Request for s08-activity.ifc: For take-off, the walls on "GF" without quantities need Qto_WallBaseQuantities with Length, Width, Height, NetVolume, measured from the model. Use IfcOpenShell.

First a look at what the model holds.

```python
import ifcopenshell
import ifcopenshell.util.element
import ifcopenshell.util.unit

model = ifcopenshell.open("s08-activity.ifc")
print(model.schema)
for unit_type in ("LENGTHUNIT", "AREAUNIT", "VOLUMEUNIT"):
    print(unit_type, ifcopenshell.util.unit.calculate_unit_scale(model, unit_type))
storey = next(s for s in model.by_type("IfcBuildingStorey") if s.Name == "GF")
walls = [e for e in ifcopenshell.util.element.get_decomposition(storey) if e.is_a("IfcWall")]
for e in sorted(walls, key=lambda e: e.id()):
    print(e.id(), e.is_a(), e.Name, list(ifcopenshell.util.element.get_psets(e, qtos_only=True)), sep=" | ")
```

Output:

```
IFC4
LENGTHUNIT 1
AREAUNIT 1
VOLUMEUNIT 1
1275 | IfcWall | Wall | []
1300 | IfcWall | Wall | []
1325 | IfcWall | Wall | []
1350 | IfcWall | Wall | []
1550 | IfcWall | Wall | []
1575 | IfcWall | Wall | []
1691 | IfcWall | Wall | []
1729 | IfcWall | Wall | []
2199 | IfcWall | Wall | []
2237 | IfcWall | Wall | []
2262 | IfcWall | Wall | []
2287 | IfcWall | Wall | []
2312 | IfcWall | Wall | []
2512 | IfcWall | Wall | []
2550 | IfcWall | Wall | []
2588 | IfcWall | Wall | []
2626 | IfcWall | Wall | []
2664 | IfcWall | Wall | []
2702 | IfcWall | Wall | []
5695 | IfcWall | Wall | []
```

```python
import ifcopenshell
import ifcopenshell.api.pset
import ifcopenshell.geom
import ifcopenshell.util.element
import ifcopenshell.util.shape
import ifcopenshell.util.unit

model = ifcopenshell.open("s08-activity.ifc")
unit_scale = ifcopenshell.util.unit.calculate_unit_scale(model)
volume_scale = ifcopenshell.util.unit.calculate_unit_scale(model, "VOLUMEUNIT")
settings = ifcopenshell.geom.settings()

storey = next(s for s in model.by_type("IfcBuildingStorey") if s.Name == "GF")
walls = [e for e in ifcopenshell.util.element.get_decomposition(storey) if e.is_a("IfcWall")]

for e in sorted(walls, key=lambda e: e.id()):
    if ifcopenshell.util.element.get_psets(e, qtos_only=True, should_inherit=False):
        continue
    # Geometry comes back in metres, in the element's own axes.
    shape = ifcopenshell.geom.create_shape(settings, e)
    values = {
        "Length": ifcopenshell.util.shape.get_x(shape.geometry) / unit_scale,
        "Width": ifcopenshell.util.shape.get_y(shape.geometry) / unit_scale,
        "Height": ifcopenshell.util.shape.get_z(shape.geometry) / unit_scale,
        "NetVolume": ifcopenshell.util.shape.get_volume(shape.geometry) / volume_scale,
    }
    qto = ifcopenshell.api.pset.add_qto(model, product=e, name="Qto_WallBaseQuantities")
    ifcopenshell.api.pset.edit_qto(model, qto=qto, properties=values)
    print(e.id(), {k: round(v, 3) for k, v in values.items()})

model.write("s08-activity_rev.ifc")
```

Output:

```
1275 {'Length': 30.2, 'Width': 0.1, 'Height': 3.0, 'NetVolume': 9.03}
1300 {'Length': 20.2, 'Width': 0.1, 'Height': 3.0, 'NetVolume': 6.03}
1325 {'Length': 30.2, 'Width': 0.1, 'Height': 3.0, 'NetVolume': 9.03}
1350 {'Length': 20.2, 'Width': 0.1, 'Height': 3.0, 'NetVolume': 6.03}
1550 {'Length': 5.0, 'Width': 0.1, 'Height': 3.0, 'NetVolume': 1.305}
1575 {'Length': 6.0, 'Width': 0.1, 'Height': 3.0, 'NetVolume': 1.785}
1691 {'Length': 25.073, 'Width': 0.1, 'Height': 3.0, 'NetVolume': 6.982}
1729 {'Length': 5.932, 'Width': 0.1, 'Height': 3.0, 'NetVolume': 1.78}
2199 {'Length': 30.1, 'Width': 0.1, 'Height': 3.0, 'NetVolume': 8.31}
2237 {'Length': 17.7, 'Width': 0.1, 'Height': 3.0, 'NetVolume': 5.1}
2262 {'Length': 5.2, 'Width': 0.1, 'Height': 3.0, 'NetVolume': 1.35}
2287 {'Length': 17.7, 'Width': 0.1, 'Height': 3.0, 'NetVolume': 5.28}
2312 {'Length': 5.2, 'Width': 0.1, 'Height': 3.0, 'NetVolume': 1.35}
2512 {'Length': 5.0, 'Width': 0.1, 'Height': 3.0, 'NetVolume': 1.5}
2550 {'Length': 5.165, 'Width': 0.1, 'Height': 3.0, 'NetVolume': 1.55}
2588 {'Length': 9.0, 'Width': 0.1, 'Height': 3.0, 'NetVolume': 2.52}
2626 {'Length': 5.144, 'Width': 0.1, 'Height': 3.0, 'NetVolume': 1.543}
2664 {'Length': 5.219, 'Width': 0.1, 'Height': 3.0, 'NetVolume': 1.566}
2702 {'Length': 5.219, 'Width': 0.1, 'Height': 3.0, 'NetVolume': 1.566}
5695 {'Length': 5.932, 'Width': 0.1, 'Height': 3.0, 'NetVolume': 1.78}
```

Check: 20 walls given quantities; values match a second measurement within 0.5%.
